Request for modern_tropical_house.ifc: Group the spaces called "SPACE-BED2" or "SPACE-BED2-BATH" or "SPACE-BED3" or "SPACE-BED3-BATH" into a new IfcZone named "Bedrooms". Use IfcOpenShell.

First a look at what the model holds.

```python
import ifcopenshell

model = ifcopenshell.open("modern_tropical_house.ifc")
print(model.schema)
seen = {}
for space in model.by_type("IfcSpace"):
    seen[space.Name] = seen.get(space.Name, 0) + 1
for name, count in sorted(seen.items(), key=str):
    print(count, "x", name)
print("zones:", [z.Name for z in model.by_type("IfcZone")][:20])
```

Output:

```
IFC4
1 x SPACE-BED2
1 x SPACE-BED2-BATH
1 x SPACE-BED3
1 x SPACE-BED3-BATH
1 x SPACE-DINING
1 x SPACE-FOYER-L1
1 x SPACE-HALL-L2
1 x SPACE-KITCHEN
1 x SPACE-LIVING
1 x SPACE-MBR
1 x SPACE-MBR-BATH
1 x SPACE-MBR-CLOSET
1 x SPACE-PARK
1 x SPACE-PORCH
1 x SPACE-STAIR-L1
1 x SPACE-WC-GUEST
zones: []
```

```python
import ifcopenshell
import ifcopenshell.api.group
import ifcopenshell.api.root

model = ifcopenshell.open("modern_tropical_house.ifc")

names = {"SPACE-BED2", "SPACE-BED2-BATH", "SPACE-BED3", "SPACE-BED3-BATH"}
spaces = [s for s in model.by_type("IfcSpace") if s.Name in names]

zone = ifcopenshell.api.root.create_entity(model, ifc_class="IfcZone", name="Bedrooms")
ifcopenshell.api.group.assign_group(model, products=spaces, group=zone)
print(len(spaces), "spaces in", zone.Name)

model.write("modern_tropical_house_v2.ifc")
```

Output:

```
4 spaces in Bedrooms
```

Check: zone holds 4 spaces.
